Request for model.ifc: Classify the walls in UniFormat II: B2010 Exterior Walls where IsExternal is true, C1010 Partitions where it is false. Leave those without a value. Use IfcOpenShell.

First a look at what the model holds.

```python
import ifcopenshell
import ifcopenshell.util.element

model = ifcopenshell.open("model.ifc")
print(model.schema)
print("classifications:", [c.Name for c in model.by_type("IfcClassification")])
values = [ifcopenshell.util.element.get_pset(e, "Pset_WallCommon", "IsExternal") for e in model.by_type("IfcWall")]
for value in (True, False, None):
    print("IsExternal", value, values.count(value))
```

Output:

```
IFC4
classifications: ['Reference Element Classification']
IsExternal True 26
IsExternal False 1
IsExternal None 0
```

```python
import ifcopenshell
import ifcopenshell.api.classification
import ifcopenshell.util.element

model = ifcopenshell.open("model.ifc")

system = ifcopenshell.api.classification.add_classification(model, classification="UniFormat II")

walls = model.by_type("IfcWall")
external = {e: ifcopenshell.util.element.get_pset(e, "Pset_WallCommon", "IsExternal") for e in walls}
for flag, code, name in ((True, "B2010", "Exterior Walls"), (False, "C1010", "Partitions")):
    products = [e for e in walls if external[e] is flag]
    ifcopenshell.api.classification.add_reference(
        model, products=products, classification=system, identification=code, name=name
    )
    print(code, len(products))

model.write("model_rev.ifc")
```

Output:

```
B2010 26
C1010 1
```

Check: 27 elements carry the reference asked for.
